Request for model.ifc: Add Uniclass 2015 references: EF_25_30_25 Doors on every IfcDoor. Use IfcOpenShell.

First a look at what the model holds.

```python
import ifcopenshell

model = ifcopenshell.open("model.ifc")
print(model.schema)
print("classifications:", [c.Name for c in model.by_type("IfcClassification")])
for ifc_class in ("IfcDoor", "IfcRoof", "IfcStair", "IfcWall", "IfcWindow"):
    print(ifc_class, len(model.by_type(ifc_class)))
```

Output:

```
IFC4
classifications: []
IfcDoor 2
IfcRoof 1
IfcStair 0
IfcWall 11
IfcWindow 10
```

```python
import ifcopenshell
import ifcopenshell.api.classification

model = ifcopenshell.open("model.ifc")

system = ifcopenshell.api.classification.add_classification(model, classification="Uniclass 2015")

codes = {
    "IfcDoor": ("EF_25_30_25", "Doors"),
}
for ifc_class, (code, name) in codes.items():
    products = model.by_type(ifc_class)
    ifcopenshell.api.classification.add_reference(
        model, products=products, classification=system, identification=code, name=name
    )
    print(code, len(products))

model.write("model_v2.ifc")
```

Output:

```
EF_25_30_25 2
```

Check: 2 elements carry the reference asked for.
